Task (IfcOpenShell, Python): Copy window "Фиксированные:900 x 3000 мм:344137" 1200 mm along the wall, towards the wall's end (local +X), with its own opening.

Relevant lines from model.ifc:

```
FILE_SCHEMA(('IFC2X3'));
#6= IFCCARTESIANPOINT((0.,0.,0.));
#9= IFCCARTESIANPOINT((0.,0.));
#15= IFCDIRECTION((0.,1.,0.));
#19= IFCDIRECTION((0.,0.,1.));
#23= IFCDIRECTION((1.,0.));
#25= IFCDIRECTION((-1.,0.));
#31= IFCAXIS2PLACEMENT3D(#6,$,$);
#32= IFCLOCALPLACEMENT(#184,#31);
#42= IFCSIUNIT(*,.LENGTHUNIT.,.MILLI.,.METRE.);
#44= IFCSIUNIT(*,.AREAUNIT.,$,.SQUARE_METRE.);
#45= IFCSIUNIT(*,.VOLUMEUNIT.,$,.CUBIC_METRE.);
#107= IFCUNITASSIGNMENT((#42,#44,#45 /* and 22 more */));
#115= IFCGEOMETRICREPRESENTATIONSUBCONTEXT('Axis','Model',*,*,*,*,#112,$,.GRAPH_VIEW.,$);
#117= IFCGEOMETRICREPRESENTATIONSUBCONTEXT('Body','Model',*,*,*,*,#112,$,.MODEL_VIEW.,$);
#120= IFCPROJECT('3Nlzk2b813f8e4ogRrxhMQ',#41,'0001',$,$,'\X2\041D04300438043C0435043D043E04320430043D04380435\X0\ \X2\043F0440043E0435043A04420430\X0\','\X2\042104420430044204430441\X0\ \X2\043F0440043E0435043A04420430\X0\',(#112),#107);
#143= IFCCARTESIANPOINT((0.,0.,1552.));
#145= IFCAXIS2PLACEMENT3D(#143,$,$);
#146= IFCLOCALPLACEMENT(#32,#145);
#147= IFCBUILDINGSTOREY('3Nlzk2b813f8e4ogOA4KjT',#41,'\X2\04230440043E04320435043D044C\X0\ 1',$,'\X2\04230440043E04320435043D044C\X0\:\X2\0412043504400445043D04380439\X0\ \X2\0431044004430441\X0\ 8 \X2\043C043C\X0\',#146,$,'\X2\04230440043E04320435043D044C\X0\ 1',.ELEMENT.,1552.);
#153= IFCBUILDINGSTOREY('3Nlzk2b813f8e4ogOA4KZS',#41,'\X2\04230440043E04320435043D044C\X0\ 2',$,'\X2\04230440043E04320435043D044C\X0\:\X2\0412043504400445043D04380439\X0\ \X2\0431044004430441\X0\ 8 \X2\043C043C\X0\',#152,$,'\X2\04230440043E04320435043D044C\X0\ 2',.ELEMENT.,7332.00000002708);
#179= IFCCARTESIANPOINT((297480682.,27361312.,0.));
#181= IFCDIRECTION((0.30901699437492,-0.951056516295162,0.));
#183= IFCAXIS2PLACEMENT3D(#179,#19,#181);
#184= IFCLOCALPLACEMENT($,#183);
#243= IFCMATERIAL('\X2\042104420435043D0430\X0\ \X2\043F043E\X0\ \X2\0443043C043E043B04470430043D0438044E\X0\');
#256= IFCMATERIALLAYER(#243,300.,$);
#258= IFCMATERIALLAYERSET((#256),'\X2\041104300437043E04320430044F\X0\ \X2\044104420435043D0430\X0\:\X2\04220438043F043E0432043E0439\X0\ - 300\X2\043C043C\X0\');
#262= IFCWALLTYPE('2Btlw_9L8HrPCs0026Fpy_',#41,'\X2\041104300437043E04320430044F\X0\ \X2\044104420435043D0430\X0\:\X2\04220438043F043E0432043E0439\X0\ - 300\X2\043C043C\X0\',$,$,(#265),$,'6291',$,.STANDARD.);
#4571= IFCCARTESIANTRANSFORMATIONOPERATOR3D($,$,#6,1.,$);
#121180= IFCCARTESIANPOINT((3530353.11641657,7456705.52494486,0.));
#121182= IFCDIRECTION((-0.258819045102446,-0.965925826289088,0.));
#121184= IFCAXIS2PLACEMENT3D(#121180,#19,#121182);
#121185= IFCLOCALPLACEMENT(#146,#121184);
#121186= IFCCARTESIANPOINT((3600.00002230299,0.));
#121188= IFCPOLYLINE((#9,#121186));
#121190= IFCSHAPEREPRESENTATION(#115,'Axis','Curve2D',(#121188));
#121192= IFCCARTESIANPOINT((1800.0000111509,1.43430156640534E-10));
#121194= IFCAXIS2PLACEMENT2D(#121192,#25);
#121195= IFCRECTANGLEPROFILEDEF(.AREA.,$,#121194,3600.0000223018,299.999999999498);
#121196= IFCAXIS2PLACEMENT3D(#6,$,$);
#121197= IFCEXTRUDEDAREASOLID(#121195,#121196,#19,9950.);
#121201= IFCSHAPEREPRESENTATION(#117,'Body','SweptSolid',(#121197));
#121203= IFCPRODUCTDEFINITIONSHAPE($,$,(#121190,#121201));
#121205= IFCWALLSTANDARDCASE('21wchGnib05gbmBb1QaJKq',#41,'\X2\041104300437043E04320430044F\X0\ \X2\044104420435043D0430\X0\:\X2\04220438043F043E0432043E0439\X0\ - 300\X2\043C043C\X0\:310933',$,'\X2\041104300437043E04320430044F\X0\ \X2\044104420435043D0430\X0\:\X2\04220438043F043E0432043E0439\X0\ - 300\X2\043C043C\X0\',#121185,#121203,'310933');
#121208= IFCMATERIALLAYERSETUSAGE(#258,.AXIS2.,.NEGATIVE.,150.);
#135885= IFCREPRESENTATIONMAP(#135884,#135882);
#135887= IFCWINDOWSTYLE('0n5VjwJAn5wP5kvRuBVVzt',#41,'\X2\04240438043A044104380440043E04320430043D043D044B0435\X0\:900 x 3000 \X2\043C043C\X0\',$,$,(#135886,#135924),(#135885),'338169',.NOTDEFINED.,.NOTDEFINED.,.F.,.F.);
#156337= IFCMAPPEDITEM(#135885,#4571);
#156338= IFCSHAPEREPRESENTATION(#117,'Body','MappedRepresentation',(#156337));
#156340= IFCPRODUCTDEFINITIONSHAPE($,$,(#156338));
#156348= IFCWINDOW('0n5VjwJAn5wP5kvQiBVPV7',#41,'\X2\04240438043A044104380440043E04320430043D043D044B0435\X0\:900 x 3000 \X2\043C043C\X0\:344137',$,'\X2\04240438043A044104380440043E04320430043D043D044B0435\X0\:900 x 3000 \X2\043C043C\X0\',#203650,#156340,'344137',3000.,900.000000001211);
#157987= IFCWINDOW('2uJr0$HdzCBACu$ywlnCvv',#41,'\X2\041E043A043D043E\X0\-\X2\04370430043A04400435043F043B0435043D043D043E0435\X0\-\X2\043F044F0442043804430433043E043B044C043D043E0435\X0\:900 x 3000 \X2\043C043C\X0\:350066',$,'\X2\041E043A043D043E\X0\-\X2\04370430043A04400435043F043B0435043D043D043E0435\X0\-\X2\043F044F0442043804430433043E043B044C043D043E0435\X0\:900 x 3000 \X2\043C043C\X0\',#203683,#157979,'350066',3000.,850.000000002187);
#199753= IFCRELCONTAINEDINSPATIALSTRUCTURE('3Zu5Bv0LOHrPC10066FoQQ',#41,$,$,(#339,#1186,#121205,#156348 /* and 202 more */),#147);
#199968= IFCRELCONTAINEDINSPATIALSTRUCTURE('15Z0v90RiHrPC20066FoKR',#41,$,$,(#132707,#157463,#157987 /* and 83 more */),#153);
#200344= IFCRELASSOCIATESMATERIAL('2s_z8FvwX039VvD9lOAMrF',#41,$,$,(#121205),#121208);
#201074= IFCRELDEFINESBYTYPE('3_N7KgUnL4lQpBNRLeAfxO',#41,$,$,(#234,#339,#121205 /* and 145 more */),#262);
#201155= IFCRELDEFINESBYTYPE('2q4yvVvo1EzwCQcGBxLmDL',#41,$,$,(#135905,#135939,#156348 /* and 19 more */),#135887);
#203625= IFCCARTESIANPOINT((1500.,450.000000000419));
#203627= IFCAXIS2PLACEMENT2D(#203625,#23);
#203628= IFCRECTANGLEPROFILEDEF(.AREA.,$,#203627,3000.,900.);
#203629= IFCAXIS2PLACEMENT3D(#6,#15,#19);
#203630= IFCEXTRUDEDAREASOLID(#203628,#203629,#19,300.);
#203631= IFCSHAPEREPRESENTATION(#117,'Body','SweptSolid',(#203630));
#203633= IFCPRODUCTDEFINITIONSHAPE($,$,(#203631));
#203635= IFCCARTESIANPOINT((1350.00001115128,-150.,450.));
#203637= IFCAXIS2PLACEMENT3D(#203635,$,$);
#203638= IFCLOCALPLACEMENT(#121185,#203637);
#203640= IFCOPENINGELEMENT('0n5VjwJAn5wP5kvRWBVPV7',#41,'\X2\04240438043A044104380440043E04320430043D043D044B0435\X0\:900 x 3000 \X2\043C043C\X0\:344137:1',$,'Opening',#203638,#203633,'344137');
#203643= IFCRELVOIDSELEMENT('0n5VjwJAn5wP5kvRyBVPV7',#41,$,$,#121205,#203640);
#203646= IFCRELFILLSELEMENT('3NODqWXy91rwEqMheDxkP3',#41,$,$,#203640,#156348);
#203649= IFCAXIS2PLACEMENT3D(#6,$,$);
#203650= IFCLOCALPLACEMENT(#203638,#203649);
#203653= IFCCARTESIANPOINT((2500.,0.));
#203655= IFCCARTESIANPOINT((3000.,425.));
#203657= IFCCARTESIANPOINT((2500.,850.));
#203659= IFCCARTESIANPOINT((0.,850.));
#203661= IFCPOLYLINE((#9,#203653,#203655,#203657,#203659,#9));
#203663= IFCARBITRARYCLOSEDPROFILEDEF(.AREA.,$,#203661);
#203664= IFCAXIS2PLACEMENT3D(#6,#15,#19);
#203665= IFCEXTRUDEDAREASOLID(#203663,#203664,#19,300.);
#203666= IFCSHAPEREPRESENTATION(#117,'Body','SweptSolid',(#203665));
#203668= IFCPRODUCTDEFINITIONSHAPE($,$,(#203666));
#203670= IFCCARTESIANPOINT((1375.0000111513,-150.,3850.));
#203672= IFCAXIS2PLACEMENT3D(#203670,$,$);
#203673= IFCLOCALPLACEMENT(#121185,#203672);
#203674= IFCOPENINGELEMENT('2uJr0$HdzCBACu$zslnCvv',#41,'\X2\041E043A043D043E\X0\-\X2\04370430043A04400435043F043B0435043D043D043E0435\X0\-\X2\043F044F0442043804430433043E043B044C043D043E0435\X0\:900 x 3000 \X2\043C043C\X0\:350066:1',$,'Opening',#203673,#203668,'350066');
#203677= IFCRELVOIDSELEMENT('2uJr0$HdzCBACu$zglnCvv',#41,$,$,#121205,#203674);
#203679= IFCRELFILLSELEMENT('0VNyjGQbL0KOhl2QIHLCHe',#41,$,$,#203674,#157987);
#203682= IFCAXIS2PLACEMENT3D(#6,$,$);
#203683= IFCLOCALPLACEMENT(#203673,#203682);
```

```python
import ifcopenshell
import ifcopenshell.api.feature
import ifcopenshell.api.geometry
import ifcopenshell.api.root
import ifcopenshell.geom
import ifcopenshell.util.element
import ifcopenshell.util.placement
import ifcopenshell.util.shape

model = ifcopenshell.open("model.ifc")
settings = ifcopenshell.geom.settings()


def volume(element):
    """Net volume in cubic metres, openings subtracted."""
    shape = ifcopenshell.geom.create_shape(settings, element)
    return ifcopenshell.util.shape.get_volume(shape.geometry)


def reuse_history(source, copy):
    """copy_class also copies each property set's owner history, people and application; keep the originals."""
    for rel in copy.IsDefinedBy:
        if rel.is_a("IfcRelDefinesByProperties") and (history := rel.RelatingPropertyDefinition.OwnerHistory):
            rel.RelatingPropertyDefinition.OwnerHistory = source.OwnerHistory
            ifcopenshell.util.element.remove_deep2(model, history)


window = model.by_guid("0n5VjwJAn5wP5kvQiBVPV7")
opening = window.FillsVoids[0].RelatingOpeningElement
wall = opening.VoidsElements[0].RelatingBuildingElement
before = volume(wall)
shift = ifcopenshell.util.placement.get_local_placement(wall.ObjectPlacement)[:3, 0] * 1200.0

# copy_class copies the void relationship, type, container and properties, but no geometry.
new_opening = ifcopenshell.api.root.copy_class(model, product=opening)
new_opening.Representation = ifcopenshell.util.element.copy_deep(
    model, opening.Representation, exclude=["IfcGeometricRepresentationContext", "IfcRepresentationMap"]
)
new_opening.Name = "Фиксированные:900 x 3000 мм"
new_opening.Tag = None
new_window = ifcopenshell.api.root.copy_class(model, product=window)
new_window.Representation = ifcopenshell.util.element.copy_deep(
    model, window.Representation, exclude=["IfcGeometricRepresentationContext", "IfcRepresentationMap"]
)
new_window.Name = "Фиксированные:900 x 3000 мм"
new_window.Tag = None
reuse_history(window, new_window)
fills = ifcopenshell.api.feature.add_filling(model, opening=new_opening, element=new_window)
fills.OwnerHistory = new_window.OwnerHistory  # required in IFC2X3

for old, new in ((opening, new_opening), (window, new_window)):
    matrix = ifcopenshell.util.placement.get_local_placement(old.ObjectPlacement)
    matrix[:3, 3] += shift
    ifcopenshell.api.geometry.edit_object_placement(model, product=new, matrix=matrix, is_si=False)

after = volume(wall)

print(f"wall volume {before:.3f} -> {after:.3f} m3")

model.write("model_updated.ifc")
```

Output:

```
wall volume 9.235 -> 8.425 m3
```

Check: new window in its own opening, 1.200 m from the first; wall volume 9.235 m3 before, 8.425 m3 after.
